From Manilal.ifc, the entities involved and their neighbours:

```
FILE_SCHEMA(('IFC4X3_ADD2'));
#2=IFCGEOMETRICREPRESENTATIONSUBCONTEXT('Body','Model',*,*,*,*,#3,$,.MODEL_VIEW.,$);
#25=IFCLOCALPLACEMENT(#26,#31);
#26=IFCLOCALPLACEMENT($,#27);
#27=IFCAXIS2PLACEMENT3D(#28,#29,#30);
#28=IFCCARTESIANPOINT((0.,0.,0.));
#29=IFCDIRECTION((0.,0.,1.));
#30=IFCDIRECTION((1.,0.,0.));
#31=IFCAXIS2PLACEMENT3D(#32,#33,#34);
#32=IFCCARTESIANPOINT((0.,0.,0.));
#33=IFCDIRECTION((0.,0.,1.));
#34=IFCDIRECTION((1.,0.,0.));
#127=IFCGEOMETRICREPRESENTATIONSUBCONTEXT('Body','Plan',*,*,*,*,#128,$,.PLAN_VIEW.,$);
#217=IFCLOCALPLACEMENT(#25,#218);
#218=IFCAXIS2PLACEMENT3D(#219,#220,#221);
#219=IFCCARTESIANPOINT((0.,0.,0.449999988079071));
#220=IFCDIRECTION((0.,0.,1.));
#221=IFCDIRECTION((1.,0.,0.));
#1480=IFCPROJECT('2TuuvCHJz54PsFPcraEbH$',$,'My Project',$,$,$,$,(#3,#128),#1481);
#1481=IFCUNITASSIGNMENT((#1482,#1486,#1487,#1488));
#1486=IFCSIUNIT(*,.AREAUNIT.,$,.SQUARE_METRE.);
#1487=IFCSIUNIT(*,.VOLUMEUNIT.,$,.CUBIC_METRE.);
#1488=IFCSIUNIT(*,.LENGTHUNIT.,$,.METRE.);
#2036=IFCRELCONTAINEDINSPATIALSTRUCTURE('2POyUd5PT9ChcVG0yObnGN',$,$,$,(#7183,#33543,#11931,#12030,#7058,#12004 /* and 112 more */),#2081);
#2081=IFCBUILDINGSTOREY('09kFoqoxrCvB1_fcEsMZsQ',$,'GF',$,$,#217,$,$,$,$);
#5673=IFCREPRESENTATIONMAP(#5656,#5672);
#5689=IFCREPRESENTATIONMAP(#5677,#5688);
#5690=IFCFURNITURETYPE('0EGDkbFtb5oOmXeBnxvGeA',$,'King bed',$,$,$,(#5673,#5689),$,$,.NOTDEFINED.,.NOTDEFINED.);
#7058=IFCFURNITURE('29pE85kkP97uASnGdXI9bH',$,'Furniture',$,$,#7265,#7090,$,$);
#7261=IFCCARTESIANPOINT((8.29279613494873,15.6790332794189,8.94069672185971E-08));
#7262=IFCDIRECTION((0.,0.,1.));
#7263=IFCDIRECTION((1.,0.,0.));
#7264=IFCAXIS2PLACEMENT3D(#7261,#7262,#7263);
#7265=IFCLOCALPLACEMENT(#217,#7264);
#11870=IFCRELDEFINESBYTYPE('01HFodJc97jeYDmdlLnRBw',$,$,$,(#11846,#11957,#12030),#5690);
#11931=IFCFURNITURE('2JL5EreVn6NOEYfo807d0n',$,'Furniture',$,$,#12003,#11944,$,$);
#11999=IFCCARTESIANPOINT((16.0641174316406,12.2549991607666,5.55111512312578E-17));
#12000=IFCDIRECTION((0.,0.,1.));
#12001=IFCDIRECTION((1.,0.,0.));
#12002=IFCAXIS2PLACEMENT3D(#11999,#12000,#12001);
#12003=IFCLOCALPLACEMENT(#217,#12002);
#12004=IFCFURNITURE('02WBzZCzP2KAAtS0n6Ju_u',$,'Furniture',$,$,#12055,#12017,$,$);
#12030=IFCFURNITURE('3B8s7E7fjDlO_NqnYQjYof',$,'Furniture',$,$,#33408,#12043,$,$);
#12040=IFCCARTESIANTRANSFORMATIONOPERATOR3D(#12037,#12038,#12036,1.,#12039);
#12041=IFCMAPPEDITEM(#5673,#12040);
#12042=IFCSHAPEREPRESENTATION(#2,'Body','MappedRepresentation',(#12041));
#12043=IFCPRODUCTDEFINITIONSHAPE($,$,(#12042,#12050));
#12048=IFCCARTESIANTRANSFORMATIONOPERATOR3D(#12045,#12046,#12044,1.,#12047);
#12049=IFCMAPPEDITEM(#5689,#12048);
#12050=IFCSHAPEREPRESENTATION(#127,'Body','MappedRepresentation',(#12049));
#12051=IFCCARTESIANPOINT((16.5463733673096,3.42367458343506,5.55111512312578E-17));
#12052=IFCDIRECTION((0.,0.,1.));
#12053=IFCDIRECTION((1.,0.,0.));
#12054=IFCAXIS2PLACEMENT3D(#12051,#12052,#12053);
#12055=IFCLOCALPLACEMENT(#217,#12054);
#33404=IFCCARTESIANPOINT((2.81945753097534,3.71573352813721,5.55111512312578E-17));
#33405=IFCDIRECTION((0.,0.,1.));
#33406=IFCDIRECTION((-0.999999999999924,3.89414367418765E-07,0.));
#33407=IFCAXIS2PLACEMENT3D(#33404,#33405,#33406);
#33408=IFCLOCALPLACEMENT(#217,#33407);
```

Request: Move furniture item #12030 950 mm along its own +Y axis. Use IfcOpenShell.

```python
import ifcopenshell
import ifcopenshell.api.geometry
import ifcopenshell.util.placement
import ifcopenshell.util.unit

model = ifcopenshell.open("Manilal.ifc")
unit_scale = ifcopenshell.util.unit.calculate_unit_scale(model)

item = model.by_guid("3B8s7E7fjDlO_NqnYQjYof")
matrix = ifcopenshell.util.placement.get_local_placement(item.ObjectPlacement)
matrix[:3, 3] += matrix[:3, 1] * 0.95 / unit_scale
ifcopenshell.api.geometry.edit_object_placement(model, product=item, matrix=matrix, is_si=False)

print(ifcopenshell.util.placement.get_local_placement(item.ObjectPlacement).round(3) + 0.0)

model.write("Manilal_edited.ifc")
```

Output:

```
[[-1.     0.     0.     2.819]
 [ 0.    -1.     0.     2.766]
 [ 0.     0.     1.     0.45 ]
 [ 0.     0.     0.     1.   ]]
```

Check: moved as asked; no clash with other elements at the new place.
